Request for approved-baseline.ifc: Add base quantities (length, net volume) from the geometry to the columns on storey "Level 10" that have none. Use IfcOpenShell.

First a look at what the model holds.

```python
import ifcopenshell
import ifcopenshell.util.element
import ifcopenshell.util.unit

model = ifcopenshell.open("approved-baseline.ifc")
print(model.schema)
for unit_type in ("LENGTHUNIT", "AREAUNIT", "VOLUMEUNIT"):
    print(unit_type, ifcopenshell.util.unit.calculate_unit_scale(model, unit_type))
storey = next(s for s in model.by_type("IfcBuildingStorey") if s.Name == "Level 10")
columns = [e for e in ifcopenshell.util.element.get_decomposition(storey) if e.is_a("IfcColumn")]
for e in sorted(columns, key=lambda e: e.id()):
    print(e.id(), e.is_a(), e.Name, list(ifcopenshell.util.element.get_psets(e, qtos_only=True)), sep=" | ")
```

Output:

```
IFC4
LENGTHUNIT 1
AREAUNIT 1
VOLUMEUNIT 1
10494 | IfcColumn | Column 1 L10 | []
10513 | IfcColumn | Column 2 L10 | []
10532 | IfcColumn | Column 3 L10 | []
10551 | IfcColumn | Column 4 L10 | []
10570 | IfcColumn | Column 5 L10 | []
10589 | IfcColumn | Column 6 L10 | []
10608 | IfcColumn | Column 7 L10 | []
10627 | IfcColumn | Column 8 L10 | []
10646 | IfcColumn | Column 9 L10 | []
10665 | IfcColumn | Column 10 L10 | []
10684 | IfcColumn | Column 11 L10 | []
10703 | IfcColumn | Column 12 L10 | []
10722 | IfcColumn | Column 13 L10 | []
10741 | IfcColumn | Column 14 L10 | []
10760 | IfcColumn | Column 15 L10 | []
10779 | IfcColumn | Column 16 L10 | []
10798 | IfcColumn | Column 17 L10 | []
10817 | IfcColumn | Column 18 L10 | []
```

```python
import ifcopenshell
import ifcopenshell.api.pset
import ifcopenshell.geom
import ifcopenshell.util.element
import ifcopenshell.util.shape
import ifcopenshell.util.unit

model = ifcopenshell.open("approved-baseline.ifc")
unit_scale = ifcopenshell.util.unit.calculate_unit_scale(model)
volume_scale = ifcopenshell.util.unit.calculate_unit_scale(model, "VOLUMEUNIT")
settings = ifcopenshell.geom.settings()

storey = next(s for s in model.by_type("IfcBuildingStorey") if s.Name == "Level 10")
columns = [e for e in ifcopenshell.util.element.get_decomposition(storey) if e.is_a("IfcColumn")]

for e in sorted(columns, key=lambda e: e.id()):
    if ifcopenshell.util.element.get_psets(e, qtos_only=True, should_inherit=False):
        continue
    # Geometry comes back in metres, in the element's own axes.
    shape = ifcopenshell.geom.create_shape(settings, e)
    values = {
        "Length": ifcopenshell.util.shape.get_z(shape.geometry) / unit_scale,
        "NetVolume": ifcopenshell.util.shape.get_volume(shape.geometry) / volume_scale,
    }
    qto = ifcopenshell.api.pset.add_qto(model, product=e, name="Qto_ColumnBaseQuantities")
    ifcopenshell.api.pset.edit_qto(model, qto=qto, properties=values)
    print(e.id(), {k: round(v, 3) for k, v in values.items()})

model.write("approved-baseline_v2.ifc")
```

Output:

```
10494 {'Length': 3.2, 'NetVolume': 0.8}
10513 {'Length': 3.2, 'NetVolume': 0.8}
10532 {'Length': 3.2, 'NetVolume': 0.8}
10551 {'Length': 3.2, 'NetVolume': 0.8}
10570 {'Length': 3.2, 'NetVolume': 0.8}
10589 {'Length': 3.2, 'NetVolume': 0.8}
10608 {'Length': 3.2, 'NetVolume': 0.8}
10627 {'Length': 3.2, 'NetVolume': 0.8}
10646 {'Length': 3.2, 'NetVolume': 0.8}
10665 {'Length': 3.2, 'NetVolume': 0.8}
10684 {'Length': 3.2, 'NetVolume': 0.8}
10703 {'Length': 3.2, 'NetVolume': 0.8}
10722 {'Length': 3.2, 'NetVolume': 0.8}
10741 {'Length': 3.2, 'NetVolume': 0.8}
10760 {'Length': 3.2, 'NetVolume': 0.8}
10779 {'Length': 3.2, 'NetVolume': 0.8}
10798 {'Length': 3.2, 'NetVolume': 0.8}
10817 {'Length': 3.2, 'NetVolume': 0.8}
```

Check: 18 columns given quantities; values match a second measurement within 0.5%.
